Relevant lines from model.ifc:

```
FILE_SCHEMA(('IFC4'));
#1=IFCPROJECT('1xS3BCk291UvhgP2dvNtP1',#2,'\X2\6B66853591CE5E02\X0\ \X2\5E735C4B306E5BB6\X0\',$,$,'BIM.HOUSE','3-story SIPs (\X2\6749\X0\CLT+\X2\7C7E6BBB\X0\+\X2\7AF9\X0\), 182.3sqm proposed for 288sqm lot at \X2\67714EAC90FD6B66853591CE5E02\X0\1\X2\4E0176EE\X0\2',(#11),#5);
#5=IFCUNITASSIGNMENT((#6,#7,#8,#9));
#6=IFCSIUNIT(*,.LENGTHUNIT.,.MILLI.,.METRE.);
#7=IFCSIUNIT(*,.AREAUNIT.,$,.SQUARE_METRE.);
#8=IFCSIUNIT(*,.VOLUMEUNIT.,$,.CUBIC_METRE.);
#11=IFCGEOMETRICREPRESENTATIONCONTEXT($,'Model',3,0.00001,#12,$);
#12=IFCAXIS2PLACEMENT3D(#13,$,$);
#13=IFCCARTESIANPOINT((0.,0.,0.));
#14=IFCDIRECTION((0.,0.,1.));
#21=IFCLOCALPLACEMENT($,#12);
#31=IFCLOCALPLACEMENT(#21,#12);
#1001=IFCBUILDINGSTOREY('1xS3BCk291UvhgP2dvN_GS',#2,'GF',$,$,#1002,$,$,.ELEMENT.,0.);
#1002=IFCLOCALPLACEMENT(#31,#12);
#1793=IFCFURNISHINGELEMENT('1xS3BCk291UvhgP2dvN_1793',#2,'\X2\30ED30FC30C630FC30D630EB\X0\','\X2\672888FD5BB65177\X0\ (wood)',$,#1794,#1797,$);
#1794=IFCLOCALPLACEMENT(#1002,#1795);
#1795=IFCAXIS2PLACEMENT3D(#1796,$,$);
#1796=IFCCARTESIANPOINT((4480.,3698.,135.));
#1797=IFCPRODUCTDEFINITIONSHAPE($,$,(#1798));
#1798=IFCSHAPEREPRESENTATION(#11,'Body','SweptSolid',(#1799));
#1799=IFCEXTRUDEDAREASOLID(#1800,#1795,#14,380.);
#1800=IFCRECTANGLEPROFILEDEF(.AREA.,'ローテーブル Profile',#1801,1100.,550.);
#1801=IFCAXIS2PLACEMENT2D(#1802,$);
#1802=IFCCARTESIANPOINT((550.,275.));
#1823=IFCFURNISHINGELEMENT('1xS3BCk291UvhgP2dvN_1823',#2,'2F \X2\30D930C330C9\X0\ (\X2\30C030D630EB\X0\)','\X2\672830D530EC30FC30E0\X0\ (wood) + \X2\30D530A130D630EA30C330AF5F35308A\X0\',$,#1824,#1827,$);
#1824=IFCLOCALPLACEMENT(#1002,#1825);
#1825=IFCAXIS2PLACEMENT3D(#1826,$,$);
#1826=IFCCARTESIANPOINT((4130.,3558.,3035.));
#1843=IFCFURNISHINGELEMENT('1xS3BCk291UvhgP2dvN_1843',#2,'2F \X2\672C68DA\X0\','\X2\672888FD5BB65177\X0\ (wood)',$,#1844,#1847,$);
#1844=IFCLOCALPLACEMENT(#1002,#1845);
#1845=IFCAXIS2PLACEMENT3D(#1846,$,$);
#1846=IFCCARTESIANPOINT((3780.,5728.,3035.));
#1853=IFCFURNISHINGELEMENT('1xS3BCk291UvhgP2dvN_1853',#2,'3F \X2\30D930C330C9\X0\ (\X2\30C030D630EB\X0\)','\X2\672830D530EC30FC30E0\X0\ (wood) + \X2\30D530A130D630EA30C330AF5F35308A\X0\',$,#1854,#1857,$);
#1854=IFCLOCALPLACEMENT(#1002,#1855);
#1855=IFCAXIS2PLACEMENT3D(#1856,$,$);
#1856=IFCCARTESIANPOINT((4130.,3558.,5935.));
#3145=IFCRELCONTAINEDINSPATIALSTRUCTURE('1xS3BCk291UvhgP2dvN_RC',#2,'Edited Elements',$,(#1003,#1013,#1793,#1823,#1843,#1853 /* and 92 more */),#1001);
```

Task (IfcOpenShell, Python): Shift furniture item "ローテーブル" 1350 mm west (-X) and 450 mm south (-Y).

```python
import ifcopenshell
import ifcopenshell.api.geometry
import ifcopenshell.util.placement
import ifcopenshell.util.unit

model = ifcopenshell.open("model.ifc")
unit_scale = ifcopenshell.util.unit.calculate_unit_scale(model)

item = model.by_guid("1xS3BCk291UvhgP2dvN_1793")
matrix = ifcopenshell.util.placement.get_local_placement(item.ObjectPlacement)
matrix[0, 3] -= 1.35 / unit_scale
matrix[1, 3] -= 0.45 / unit_scale
ifcopenshell.api.geometry.edit_object_placement(model, product=item, matrix=matrix, is_si=False)

print(ifcopenshell.util.placement.get_local_placement(item.ObjectPlacement).round(3) + 0.0)

model.write("model_updated.ifc")
```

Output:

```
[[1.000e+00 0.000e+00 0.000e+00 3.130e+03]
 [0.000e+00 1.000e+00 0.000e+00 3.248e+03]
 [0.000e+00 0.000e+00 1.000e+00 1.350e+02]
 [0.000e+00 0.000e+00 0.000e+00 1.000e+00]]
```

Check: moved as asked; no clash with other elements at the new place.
